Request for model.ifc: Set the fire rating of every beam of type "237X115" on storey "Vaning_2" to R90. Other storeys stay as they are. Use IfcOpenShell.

First a look at what the model holds.

```python
import ifcopenshell
import ifcopenshell.util.element

model = ifcopenshell.open("model.ifc")
print(model.schema)
storey = next(s for s in model.by_type("IfcBuildingStorey") if s.Name == "Vaning_2")
beams = [e for e in ifcopenshell.util.element.get_decomposition(storey) if e.is_a("IfcBeam")]
seen = {}
for e in beams:
    element_type = ifcopenshell.util.element.get_type(e)
    key = (element_type.Name if element_type != e and element_type else None, ifcopenshell.util.element.get_pset(e, "Pset_BeamCommon", "FireRating"))
    seen[key] = seen.get(key, 0) + 1
for (name, value), count in sorted(seen.items(), key=str):
    print(count, "x", name, "|", value)
```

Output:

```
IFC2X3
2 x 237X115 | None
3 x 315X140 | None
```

```python
import ifcopenshell
import ifcopenshell.api.pset
import ifcopenshell.util.element

model = ifcopenshell.open("model.ifc")

storey = next(s for s in model.by_type("IfcBuildingStorey") if s.Name == "Vaning_2")
beams = [e for e in ifcopenshell.util.element.get_decomposition(storey) if e.is_a("IfcBeam")]

count = 0
for e in beams:
    element_type = ifcopenshell.util.element.get_type(e)
    if element_type in (None, e) or element_type.Name != "237X115":
        continue
    # add_pset returns the element's existing set when there is one.
    pset = ifcopenshell.api.pset.add_pset(model, product=e, name="Pset_BeamCommon")
    ifcopenshell.api.pset.edit_pset(model, pset=pset, properties={"FireRating": "R90"})
    count += 1

print(count, "beams updated")

model.write("model_rev.ifc")
```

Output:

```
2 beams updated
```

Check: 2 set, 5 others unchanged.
